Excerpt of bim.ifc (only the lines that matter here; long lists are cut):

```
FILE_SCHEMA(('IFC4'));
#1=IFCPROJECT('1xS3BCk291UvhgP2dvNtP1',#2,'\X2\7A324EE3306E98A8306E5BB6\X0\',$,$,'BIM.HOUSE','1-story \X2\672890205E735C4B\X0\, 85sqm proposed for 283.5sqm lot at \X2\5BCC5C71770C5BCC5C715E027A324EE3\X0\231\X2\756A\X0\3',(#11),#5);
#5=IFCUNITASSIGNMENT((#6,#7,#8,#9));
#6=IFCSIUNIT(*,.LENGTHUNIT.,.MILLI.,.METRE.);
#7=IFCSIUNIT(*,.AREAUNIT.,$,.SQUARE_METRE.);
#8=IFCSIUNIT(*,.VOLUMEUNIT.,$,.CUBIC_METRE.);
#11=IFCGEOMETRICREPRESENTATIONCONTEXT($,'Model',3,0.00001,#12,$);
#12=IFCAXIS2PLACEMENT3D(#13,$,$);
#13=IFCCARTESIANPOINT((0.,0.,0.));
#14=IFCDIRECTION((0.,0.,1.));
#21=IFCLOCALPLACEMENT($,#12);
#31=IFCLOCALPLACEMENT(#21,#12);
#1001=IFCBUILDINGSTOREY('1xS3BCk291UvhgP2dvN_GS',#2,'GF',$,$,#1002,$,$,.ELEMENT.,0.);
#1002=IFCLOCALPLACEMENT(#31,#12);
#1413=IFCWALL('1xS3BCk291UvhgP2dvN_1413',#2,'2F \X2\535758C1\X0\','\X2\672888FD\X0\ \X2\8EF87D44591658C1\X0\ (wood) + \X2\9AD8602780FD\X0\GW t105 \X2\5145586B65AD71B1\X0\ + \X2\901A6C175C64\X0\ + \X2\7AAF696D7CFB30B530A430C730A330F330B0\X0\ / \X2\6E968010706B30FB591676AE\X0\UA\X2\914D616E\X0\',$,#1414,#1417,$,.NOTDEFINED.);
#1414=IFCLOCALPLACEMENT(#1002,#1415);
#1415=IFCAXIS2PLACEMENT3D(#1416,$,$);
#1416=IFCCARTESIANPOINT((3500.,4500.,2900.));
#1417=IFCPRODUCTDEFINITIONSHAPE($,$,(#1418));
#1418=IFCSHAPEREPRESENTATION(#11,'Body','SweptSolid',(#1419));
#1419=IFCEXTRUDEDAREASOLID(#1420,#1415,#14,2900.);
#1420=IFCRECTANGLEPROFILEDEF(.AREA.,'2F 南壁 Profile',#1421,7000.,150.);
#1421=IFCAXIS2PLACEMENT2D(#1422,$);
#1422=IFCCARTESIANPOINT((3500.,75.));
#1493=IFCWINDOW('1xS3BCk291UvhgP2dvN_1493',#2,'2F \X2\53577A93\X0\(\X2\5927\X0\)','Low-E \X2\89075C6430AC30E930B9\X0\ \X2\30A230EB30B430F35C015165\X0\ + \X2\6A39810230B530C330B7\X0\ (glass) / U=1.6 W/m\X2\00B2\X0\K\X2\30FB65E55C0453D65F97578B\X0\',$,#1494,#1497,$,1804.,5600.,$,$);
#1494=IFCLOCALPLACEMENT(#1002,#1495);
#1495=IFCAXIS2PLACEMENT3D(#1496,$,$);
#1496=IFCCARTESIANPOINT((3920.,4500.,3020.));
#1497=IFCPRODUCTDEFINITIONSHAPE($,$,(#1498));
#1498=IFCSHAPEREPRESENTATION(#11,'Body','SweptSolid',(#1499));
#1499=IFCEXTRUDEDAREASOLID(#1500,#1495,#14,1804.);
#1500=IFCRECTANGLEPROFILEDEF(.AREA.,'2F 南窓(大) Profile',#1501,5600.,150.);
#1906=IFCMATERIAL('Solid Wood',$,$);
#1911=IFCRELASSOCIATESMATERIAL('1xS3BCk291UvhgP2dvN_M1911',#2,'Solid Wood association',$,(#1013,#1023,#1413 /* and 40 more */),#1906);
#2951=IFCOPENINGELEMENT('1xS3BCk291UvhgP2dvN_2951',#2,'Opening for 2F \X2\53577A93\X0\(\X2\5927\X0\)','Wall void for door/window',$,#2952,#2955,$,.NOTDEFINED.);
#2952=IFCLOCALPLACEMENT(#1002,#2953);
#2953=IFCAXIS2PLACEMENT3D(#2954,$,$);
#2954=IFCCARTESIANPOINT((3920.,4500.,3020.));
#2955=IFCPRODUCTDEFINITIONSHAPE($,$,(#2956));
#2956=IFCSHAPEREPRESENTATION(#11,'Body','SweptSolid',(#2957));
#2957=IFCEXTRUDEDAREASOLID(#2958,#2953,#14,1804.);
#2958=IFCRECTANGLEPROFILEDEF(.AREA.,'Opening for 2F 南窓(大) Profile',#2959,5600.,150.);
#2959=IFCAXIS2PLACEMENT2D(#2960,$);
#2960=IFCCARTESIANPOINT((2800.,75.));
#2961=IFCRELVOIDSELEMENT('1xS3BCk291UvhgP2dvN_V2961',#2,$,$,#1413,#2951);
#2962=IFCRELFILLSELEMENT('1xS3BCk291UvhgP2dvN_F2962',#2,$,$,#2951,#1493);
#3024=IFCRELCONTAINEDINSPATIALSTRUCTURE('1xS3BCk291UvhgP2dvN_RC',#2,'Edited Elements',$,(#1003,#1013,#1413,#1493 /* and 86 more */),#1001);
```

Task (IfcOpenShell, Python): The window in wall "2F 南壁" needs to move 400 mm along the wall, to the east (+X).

```python
import ifcopenshell
import ifcopenshell.api.geometry
import ifcopenshell.util.placement
import ifcopenshell.util.unit

model = ifcopenshell.open("bim.ifc")
unit_scale = ifcopenshell.util.unit.calculate_unit_scale(model)

window = model.by_id(1493)
opening = window.FillsVoids[0].RelatingOpeningElement
wall = opening.VoidsElements[0].RelatingBuildingElement

wall_matrix = ifcopenshell.util.placement.get_local_placement(wall.ObjectPlacement)
shift = wall_matrix[:3, 0] * 0.4 / unit_scale
before = ifcopenshell.util.placement.get_local_placement(window.ObjectPlacement)[:3, 3].copy()

# The window is not placed relative to its opening, so move both.
for product in (opening, window):
    matrix = ifcopenshell.util.placement.get_local_placement(product.ObjectPlacement)
    matrix[:3, 3] += shift
    ifcopenshell.api.geometry.edit_object_placement(model, product=product, matrix=matrix, is_si=False)

after = ifcopenshell.util.placement.get_local_placement(window.ObjectPlacement)[:3, 3]
print("window moved by", (after - before).round(3) + 0.0)

model.write("bim_rev.ifc")
```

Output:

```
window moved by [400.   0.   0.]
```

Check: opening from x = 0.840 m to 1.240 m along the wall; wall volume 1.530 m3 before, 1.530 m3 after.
